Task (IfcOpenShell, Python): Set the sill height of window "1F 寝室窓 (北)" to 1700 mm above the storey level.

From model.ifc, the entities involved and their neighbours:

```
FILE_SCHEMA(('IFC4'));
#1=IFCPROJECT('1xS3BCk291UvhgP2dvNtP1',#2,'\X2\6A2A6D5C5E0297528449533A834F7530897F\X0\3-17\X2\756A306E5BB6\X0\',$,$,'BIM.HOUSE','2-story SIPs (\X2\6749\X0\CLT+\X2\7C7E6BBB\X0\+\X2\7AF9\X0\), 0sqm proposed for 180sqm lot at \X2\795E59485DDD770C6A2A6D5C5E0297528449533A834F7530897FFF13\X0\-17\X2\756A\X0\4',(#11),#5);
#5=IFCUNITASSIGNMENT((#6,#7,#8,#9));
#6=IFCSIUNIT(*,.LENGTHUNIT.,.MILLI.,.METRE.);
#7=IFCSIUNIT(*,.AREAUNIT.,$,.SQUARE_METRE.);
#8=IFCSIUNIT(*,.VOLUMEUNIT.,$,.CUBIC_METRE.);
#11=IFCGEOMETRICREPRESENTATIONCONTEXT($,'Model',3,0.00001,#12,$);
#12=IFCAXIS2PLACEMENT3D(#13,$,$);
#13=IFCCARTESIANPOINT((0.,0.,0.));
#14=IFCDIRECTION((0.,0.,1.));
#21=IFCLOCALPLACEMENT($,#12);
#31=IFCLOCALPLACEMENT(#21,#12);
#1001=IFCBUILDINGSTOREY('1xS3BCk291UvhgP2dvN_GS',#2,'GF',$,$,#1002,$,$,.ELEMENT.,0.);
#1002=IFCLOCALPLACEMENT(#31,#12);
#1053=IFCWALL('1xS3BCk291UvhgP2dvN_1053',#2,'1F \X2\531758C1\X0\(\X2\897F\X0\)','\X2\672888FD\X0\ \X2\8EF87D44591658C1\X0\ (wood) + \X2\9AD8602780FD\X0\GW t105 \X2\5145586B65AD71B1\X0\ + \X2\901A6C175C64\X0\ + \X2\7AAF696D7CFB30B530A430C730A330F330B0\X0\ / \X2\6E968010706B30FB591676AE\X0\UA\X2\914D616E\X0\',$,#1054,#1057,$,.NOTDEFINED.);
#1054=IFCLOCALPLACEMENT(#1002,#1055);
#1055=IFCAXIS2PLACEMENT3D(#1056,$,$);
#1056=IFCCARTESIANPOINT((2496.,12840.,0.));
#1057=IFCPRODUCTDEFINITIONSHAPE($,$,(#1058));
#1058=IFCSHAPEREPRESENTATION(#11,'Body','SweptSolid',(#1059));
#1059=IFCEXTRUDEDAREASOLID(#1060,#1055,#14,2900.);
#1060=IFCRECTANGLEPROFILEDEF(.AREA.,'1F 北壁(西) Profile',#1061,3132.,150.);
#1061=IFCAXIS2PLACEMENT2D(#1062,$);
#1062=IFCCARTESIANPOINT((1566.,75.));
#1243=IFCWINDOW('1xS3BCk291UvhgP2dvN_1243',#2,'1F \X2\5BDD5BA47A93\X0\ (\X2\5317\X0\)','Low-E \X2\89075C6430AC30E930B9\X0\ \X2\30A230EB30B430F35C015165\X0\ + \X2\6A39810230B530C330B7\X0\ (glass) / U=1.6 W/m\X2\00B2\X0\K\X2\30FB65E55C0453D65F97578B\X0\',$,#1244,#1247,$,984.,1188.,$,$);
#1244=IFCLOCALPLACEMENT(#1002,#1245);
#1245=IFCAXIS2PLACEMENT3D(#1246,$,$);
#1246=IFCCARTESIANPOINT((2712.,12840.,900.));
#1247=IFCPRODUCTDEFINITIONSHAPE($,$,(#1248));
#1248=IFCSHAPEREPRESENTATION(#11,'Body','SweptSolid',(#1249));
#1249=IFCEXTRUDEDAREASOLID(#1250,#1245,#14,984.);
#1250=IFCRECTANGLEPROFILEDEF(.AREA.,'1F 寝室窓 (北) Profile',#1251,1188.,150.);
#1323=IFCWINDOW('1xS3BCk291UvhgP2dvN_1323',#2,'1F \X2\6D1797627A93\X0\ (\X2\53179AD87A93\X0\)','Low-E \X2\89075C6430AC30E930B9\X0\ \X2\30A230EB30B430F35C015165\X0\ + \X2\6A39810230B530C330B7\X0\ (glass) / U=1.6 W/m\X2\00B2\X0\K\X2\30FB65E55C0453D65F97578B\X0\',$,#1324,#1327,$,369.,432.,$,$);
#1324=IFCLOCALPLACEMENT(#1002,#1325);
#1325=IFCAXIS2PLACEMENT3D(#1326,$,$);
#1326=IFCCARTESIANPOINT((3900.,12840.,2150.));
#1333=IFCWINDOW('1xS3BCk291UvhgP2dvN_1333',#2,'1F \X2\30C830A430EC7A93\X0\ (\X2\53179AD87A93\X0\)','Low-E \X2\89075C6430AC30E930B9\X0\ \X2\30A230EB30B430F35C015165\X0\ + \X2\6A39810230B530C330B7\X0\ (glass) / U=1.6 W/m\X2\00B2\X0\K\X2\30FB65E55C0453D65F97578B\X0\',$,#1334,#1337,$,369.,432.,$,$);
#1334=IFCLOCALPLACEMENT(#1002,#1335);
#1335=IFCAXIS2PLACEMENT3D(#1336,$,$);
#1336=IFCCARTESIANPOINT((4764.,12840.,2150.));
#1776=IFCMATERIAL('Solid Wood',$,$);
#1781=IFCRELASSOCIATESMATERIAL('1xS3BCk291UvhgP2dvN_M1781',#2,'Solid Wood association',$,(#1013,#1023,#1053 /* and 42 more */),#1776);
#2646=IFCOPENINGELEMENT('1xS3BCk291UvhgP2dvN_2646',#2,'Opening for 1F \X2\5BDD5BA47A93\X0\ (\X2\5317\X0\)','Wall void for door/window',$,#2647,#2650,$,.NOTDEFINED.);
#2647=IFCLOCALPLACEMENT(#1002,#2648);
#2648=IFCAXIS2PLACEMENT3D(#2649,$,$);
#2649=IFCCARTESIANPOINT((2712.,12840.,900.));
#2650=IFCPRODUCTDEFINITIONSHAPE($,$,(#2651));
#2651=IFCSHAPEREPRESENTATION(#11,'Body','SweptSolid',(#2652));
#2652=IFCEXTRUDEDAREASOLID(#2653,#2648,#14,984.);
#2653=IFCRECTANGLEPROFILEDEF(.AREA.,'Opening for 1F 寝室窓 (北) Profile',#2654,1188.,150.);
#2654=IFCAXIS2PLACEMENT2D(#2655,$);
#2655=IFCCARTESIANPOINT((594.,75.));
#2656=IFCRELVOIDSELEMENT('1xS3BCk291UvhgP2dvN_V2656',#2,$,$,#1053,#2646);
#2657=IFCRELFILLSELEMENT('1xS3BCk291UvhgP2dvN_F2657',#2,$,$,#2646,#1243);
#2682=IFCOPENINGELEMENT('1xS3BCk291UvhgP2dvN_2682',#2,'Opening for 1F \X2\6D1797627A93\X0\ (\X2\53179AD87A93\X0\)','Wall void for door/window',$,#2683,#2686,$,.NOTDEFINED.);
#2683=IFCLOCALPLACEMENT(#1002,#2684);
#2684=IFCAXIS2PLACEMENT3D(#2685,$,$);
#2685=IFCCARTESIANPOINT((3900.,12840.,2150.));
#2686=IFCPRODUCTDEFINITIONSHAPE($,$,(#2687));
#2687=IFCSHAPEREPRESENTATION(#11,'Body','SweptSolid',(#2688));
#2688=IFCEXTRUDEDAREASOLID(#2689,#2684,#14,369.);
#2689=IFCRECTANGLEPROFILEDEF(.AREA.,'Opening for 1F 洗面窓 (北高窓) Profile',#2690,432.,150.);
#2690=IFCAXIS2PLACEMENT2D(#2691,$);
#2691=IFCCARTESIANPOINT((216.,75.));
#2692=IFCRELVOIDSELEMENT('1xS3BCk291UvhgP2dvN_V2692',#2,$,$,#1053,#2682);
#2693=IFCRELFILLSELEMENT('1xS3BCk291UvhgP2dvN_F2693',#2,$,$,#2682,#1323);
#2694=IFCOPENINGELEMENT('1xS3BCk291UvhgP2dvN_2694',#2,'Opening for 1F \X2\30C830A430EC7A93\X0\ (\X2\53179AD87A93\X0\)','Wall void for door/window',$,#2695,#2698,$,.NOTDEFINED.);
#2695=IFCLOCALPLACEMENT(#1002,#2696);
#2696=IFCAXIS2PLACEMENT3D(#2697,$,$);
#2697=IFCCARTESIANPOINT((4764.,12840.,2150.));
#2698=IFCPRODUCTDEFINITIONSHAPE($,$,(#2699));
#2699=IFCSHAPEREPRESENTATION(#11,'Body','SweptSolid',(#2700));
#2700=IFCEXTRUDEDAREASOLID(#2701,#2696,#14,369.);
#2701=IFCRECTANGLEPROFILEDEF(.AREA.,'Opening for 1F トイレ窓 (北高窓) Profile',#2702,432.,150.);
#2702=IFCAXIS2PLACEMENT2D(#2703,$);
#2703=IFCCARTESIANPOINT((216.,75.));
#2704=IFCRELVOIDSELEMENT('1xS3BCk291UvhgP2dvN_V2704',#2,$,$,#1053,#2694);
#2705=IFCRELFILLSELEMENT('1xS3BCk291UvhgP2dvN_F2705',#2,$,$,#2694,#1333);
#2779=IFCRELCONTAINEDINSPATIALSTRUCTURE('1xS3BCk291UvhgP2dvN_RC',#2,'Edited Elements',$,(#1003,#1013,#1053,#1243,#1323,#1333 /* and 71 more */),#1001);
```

```python
import numpy as np
import ifcopenshell
import ifcopenshell.api.geometry
import ifcopenshell.geom
import ifcopenshell.util.element
import ifcopenshell.util.placement
import ifcopenshell.util.shape
import ifcopenshell.util.unit

model = ifcopenshell.open("model.ifc")
unit_scale = ifcopenshell.util.unit.calculate_unit_scale(model)

window = model.by_id(1243)
opening = window.FillsVoids[0].RelatingOpeningElement
storey = ifcopenshell.util.element.get_container(window, ifc_class="IfcBuildingStorey")
level = ifcopenshell.util.placement.get_local_placement(storey.ObjectPlacement)[2, 3]

# The opening's origin need not be at the sill, so measure its lowest point.
shape = ifcopenshell.geom.create_shape(ifcopenshell.geom.settings(), opening)
bottom = ifcopenshell.util.shape.get_shape_bottom_elevation(shape, shape.geometry) / unit_scale
dz = level + 1700.0 - bottom

shift = np.array([0.0, 0.0, dz])
# The window is not placed relative to its opening, so move both.
for product in (opening, window):
    matrix = ifcopenshell.util.placement.get_local_placement(product.ObjectPlacement)
    matrix[:3, 3] += shift
    ifcopenshell.api.geometry.edit_object_placement(model, product=product, matrix=matrix, is_si=False)

print(f"moved by {dz * unit_scale:+.3f} m")

model.write("model_updated.ifc")
```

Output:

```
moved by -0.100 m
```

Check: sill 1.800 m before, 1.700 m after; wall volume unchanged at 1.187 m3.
